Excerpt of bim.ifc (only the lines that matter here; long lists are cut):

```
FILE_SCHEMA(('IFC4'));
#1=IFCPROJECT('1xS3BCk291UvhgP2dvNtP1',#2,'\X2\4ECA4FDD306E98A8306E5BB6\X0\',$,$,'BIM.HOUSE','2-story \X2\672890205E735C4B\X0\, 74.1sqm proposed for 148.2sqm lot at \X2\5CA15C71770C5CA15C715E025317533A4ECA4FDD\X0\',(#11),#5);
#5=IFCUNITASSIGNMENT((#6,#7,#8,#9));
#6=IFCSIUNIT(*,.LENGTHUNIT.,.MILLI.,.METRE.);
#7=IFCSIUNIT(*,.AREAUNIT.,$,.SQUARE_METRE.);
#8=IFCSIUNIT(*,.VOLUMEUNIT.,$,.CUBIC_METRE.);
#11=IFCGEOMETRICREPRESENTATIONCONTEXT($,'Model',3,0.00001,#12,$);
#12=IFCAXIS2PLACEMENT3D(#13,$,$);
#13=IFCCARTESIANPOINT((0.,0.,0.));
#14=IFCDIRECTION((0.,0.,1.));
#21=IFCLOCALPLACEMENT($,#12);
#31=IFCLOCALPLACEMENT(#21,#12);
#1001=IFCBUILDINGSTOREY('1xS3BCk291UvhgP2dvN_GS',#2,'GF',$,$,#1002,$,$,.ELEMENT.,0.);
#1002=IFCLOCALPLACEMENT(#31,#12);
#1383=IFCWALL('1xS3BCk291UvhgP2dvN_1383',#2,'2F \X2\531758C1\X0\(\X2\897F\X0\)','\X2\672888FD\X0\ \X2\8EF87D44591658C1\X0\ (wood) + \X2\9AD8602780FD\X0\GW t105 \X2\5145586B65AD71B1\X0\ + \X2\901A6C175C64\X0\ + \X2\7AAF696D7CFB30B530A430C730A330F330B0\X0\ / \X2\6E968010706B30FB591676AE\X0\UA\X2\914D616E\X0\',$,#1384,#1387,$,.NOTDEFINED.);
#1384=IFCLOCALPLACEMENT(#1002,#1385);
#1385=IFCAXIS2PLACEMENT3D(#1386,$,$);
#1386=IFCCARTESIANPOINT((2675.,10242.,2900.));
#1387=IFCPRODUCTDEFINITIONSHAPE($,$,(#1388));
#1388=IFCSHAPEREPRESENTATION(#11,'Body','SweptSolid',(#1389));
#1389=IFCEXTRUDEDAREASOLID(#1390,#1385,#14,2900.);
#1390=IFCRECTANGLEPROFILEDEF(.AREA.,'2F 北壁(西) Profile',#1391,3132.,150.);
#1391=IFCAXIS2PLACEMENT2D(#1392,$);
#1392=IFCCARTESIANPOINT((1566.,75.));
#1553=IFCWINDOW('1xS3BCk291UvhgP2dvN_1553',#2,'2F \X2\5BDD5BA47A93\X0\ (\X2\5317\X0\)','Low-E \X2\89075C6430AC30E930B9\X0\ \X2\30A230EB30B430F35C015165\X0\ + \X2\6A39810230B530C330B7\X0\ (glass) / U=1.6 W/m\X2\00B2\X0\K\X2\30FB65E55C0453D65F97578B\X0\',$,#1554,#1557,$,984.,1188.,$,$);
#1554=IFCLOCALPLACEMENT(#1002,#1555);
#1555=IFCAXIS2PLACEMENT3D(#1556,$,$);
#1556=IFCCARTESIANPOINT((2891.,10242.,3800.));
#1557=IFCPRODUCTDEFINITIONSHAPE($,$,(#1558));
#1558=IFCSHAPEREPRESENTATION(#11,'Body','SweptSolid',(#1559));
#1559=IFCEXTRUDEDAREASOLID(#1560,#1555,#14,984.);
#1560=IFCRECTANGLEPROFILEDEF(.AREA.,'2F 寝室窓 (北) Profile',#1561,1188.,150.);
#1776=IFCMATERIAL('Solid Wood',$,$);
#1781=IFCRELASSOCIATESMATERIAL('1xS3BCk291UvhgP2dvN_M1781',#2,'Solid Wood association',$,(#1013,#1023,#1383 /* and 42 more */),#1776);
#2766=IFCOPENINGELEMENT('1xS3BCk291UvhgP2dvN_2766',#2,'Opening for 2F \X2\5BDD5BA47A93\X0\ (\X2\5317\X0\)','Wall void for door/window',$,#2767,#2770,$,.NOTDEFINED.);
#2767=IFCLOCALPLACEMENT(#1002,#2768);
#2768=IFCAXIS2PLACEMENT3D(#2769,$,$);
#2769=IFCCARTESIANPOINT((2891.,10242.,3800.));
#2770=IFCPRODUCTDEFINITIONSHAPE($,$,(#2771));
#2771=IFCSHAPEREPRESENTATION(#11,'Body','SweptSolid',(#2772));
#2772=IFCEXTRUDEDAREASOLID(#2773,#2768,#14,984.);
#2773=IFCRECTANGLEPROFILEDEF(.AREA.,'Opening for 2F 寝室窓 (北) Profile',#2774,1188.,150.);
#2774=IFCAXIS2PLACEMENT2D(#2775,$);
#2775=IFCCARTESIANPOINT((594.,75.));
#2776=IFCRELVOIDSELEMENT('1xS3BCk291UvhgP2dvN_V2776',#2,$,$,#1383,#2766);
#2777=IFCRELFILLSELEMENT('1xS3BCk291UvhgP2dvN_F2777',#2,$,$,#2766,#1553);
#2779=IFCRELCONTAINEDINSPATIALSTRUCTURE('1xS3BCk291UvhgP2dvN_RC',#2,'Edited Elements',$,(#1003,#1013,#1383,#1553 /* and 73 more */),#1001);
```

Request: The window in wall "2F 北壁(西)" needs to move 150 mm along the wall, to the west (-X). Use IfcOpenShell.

```python
import ifcopenshell
import ifcopenshell.api.geometry
import ifcopenshell.util.placement

model = ifcopenshell.open("bim.ifc")

window = model.by_id(1553)
opening = window.FillsVoids[0].RelatingOpeningElement
wall = opening.VoidsElements[0].RelatingBuildingElement

wall_matrix = ifcopenshell.util.placement.get_local_placement(wall.ObjectPlacement)
shift = wall_matrix[:3, 0] * -150.0
before = ifcopenshell.util.placement.get_local_placement(window.ObjectPlacement)[:3, 3].copy()

# The window is not placed relative to its opening, so move both.
for product in (opening, window):
    matrix = ifcopenshell.util.placement.get_local_placement(product.ObjectPlacement)
    matrix[:3, 3] += shift
    ifcopenshell.api.geometry.edit_object_placement(model, product=product, matrix=matrix, is_si=False)

after = ifcopenshell.util.placement.get_local_placement(window.ObjectPlacement)[:3, 3]
print("window moved by", (after - before).round(3) + 0.0)

model.write("bim_edited.ifc")
```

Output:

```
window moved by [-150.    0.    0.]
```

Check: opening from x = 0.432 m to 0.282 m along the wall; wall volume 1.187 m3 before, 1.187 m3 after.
